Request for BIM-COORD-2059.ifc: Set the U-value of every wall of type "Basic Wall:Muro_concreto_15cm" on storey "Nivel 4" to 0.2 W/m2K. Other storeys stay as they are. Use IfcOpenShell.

First a look at what the model holds.

```python
import ifcopenshell
import ifcopenshell.util.element

model = ifcopenshell.open("BIM-COORD-2059.ifc")
print(model.schema)
storey = next(s for s in model.by_type("IfcBuildingStorey") if s.Name == "Nivel 4")
walls = [e for e in ifcopenshell.util.element.get_decomposition(storey) if e.is_a("IfcWall")]
seen = {}
for e in walls:
    element_type = ifcopenshell.util.element.get_type(e)
    key = (element_type.Name if element_type != e and element_type else None, ifcopenshell.util.element.get_pset(e, "Pset_WallCommon", "ThermalTransmittance"))
    seen[key] = seen.get(key, 0) + 1
for (name, value), count in sorted(seen.items(), key=str):
    print(count, "x", name, "|", value)
```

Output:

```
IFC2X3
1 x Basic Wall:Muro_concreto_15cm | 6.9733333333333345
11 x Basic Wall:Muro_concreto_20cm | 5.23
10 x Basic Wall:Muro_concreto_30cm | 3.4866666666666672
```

```python
import ifcopenshell
import ifcopenshell.api.pset
import ifcopenshell.util.element

model = ifcopenshell.open("BIM-COORD-2059.ifc")

storey = next(s for s in model.by_type("IfcBuildingStorey") if s.Name == "Nivel 4")
walls = [e for e in ifcopenshell.util.element.get_decomposition(storey) if e.is_a("IfcWall")]

count = 0
for e in walls:
    element_type = ifcopenshell.util.element.get_type(e)
    if element_type in (None, e) or element_type.Name != "Basic Wall:Muro_concreto_15cm":
        continue
    # add_pset returns the element's existing set when there is one.
    pset = ifcopenshell.api.pset.add_pset(model, product=e, name="Pset_WallCommon")
    ifcopenshell.api.pset.edit_pset(model, pset=pset, properties={"ThermalTransmittance": 0.2})
    count += 1

print(count, "walls updated")

model.write("BIM-COORD-2059_edited.ifc")
```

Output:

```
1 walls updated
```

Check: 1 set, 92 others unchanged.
